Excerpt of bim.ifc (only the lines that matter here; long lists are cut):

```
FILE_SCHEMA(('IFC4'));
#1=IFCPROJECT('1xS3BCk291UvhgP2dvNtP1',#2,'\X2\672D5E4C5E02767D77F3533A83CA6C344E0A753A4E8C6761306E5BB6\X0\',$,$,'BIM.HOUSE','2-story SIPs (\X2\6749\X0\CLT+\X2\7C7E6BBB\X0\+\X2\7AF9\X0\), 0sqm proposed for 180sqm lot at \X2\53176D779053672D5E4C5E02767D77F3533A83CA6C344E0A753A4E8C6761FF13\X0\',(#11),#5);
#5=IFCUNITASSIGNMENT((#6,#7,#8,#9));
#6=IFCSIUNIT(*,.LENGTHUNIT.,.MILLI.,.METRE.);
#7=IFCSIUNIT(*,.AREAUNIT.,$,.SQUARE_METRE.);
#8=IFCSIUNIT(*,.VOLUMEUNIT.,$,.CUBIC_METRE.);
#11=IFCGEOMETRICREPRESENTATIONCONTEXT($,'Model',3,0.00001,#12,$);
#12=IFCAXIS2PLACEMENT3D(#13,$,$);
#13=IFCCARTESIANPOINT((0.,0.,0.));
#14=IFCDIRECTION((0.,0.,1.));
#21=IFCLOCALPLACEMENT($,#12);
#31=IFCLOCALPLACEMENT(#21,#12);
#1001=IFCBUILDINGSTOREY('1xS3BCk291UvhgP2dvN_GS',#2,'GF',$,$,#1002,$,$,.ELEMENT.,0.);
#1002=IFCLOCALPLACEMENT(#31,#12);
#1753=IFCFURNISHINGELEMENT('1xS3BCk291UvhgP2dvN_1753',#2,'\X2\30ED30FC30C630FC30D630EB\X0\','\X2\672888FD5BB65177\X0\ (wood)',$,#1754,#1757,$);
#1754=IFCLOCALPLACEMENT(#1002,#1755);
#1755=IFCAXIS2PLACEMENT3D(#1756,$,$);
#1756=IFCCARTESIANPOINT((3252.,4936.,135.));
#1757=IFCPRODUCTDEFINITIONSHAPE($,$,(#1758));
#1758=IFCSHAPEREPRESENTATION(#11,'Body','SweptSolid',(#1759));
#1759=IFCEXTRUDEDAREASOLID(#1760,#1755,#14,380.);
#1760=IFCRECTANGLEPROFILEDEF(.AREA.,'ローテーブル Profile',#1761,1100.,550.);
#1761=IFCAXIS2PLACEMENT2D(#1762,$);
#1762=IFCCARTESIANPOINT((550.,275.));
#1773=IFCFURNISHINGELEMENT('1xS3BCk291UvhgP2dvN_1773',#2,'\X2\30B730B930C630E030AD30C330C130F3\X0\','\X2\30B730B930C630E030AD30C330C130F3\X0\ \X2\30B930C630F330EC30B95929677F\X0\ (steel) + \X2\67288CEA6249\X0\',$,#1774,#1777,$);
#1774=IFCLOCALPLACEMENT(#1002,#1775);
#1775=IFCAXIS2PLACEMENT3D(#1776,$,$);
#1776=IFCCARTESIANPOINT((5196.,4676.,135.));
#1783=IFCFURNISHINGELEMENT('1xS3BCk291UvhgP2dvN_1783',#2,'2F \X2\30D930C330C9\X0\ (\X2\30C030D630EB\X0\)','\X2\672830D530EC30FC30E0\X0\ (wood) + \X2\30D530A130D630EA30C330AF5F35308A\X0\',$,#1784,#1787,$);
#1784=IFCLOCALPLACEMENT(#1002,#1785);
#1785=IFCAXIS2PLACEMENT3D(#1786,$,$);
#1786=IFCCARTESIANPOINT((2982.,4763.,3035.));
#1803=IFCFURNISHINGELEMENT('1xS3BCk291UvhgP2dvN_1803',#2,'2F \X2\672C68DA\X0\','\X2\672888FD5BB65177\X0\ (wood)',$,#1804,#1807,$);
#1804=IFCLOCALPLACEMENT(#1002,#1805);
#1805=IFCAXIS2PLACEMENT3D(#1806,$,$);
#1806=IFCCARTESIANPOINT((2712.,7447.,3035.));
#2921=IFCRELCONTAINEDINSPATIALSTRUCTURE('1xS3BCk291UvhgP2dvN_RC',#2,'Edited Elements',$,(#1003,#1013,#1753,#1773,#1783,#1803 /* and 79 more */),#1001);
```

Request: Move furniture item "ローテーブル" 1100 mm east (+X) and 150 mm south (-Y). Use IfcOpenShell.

```python
import ifcopenshell
import ifcopenshell.api.geometry
import ifcopenshell.util.placement
import ifcopenshell.util.unit

model = ifcopenshell.open("bim.ifc")
unit_scale = ifcopenshell.util.unit.calculate_unit_scale(model)

item = model.by_id(1753)
matrix = ifcopenshell.util.placement.get_local_placement(item.ObjectPlacement)
matrix[0, 3] += 1.1 / unit_scale
matrix[1, 3] -= 0.15 / unit_scale
ifcopenshell.api.geometry.edit_object_placement(model, product=item, matrix=matrix, is_si=False)

print(ifcopenshell.util.placement.get_local_placement(item.ObjectPlacement).round(3) + 0.0)

model.write("bim_v2.ifc")
```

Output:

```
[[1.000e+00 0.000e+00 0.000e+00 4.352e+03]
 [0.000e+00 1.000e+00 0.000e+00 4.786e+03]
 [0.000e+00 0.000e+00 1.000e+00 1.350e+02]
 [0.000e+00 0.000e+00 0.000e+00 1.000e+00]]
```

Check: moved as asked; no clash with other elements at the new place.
